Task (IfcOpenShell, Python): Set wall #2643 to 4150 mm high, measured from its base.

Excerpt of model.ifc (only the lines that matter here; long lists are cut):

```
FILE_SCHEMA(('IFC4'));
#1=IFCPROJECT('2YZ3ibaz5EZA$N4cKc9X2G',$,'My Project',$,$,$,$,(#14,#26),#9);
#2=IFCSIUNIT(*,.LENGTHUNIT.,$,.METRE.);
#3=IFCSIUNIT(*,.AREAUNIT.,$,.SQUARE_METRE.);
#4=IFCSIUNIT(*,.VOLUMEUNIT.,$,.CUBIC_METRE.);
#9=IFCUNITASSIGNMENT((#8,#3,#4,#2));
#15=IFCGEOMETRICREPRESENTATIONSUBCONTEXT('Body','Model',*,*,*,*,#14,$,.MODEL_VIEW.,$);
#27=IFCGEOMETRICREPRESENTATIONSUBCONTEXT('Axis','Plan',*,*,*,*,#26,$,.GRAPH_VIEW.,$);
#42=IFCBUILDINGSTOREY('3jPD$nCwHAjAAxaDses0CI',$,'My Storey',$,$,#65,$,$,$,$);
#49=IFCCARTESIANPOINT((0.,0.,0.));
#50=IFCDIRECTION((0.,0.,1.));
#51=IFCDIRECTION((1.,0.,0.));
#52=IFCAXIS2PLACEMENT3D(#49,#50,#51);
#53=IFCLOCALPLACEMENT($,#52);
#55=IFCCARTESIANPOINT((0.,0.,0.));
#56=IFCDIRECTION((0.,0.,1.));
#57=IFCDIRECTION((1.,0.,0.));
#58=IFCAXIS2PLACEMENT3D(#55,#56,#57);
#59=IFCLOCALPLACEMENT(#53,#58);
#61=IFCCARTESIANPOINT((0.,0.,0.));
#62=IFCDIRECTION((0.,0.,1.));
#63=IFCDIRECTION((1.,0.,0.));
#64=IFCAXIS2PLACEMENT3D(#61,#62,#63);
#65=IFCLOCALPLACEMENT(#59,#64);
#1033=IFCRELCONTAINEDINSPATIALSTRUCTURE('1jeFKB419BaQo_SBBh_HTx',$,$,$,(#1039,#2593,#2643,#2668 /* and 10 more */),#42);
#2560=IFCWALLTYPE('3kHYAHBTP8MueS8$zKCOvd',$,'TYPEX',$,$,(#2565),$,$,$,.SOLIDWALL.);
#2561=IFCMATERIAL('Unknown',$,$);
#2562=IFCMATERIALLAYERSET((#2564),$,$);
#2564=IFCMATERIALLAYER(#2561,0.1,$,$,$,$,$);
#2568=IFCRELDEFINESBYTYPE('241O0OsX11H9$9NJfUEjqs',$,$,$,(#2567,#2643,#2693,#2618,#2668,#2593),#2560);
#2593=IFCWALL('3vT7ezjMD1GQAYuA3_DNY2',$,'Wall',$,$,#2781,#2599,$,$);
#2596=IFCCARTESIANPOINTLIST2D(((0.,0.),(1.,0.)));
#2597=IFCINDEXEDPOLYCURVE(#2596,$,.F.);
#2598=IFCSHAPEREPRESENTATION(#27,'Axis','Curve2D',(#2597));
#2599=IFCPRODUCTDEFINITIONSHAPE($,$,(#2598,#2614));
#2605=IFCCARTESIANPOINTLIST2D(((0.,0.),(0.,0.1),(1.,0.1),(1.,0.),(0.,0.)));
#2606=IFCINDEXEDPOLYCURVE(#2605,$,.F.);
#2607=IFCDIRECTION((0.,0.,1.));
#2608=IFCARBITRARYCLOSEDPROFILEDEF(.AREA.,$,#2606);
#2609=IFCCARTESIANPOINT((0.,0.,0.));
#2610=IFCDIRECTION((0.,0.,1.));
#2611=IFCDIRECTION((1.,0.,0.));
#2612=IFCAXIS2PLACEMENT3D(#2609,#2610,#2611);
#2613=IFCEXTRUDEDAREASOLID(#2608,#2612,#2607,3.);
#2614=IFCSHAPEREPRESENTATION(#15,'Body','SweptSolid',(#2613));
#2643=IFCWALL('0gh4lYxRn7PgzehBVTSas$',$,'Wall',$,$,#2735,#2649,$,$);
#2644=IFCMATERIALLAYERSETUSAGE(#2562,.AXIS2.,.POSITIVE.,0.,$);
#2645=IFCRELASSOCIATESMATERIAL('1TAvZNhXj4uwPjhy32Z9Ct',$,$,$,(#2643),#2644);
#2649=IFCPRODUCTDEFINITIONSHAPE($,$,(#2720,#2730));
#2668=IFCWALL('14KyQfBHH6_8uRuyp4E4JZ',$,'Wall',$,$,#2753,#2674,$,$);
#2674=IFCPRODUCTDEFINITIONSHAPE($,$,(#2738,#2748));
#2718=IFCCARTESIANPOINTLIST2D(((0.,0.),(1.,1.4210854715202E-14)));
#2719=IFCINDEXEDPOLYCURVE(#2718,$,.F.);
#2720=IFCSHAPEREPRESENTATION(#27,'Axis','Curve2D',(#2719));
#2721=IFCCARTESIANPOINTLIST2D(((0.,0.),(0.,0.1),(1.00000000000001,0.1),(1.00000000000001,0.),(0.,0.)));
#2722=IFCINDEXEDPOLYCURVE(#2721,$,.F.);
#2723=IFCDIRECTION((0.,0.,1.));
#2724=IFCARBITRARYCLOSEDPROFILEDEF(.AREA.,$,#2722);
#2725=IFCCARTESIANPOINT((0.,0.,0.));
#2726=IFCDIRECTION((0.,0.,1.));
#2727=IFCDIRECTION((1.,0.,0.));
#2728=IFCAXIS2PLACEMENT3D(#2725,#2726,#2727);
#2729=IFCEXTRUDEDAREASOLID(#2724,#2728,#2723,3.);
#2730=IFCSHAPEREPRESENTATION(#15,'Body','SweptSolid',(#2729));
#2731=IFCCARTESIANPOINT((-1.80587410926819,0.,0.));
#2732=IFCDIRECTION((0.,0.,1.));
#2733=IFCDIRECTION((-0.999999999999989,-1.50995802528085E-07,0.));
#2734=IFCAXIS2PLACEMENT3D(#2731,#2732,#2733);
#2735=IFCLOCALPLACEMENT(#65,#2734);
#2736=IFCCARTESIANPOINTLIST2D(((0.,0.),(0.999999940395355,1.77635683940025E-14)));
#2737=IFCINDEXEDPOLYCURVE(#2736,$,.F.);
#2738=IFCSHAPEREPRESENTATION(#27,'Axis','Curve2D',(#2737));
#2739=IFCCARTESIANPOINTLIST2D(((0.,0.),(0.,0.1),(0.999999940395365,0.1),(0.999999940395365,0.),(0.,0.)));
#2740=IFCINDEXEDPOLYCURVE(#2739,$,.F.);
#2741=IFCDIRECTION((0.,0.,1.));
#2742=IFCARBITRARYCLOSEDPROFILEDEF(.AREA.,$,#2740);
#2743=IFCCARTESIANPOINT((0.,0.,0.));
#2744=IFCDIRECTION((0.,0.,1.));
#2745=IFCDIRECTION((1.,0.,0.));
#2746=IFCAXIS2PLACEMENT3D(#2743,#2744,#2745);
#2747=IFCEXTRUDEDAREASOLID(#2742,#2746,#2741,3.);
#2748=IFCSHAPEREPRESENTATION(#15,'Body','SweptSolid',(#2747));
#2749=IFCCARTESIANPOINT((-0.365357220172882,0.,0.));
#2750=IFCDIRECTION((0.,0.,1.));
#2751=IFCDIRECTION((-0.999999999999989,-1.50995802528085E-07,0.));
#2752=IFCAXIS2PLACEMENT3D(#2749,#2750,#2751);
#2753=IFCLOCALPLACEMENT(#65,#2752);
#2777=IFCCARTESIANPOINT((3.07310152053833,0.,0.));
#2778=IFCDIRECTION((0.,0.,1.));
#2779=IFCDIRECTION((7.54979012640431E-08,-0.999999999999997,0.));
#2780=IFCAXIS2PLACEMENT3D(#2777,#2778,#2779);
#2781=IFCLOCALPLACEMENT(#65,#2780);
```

```python
import ifcopenshell
import ifcopenshell.geom
import ifcopenshell.util.representation
import ifcopenshell.util.shape
import ifcopenshell.util.unit

model = ifcopenshell.open("model.ifc")
unit_scale = ifcopenshell.util.unit.calculate_unit_scale(model)
settings = ifcopenshell.geom.settings()


def volume(element):
    """Net volume in cubic metres, openings subtracted."""
    shape = ifcopenshell.geom.create_shape(settings, element)
    return ifcopenshell.util.shape.get_volume(shape.geometry)


wall = model.by_guid("0gh4lYxRn7PgzehBVTSas$")
before = volume(wall)

body = ifcopenshell.util.representation.get_representation(wall, "Model", "Body")
solid = body.Items[0]
old_height = solid.Depth
solid.Depth = 4.15 / unit_scale
after = volume(wall)

print(f"height {old_height:g} -> {solid.Depth:g}, volume {before:.3f} -> {after:.3f} m3")

model.write("model_edited.ifc")
```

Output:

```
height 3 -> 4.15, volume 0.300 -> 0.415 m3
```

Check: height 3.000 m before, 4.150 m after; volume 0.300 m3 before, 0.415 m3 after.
